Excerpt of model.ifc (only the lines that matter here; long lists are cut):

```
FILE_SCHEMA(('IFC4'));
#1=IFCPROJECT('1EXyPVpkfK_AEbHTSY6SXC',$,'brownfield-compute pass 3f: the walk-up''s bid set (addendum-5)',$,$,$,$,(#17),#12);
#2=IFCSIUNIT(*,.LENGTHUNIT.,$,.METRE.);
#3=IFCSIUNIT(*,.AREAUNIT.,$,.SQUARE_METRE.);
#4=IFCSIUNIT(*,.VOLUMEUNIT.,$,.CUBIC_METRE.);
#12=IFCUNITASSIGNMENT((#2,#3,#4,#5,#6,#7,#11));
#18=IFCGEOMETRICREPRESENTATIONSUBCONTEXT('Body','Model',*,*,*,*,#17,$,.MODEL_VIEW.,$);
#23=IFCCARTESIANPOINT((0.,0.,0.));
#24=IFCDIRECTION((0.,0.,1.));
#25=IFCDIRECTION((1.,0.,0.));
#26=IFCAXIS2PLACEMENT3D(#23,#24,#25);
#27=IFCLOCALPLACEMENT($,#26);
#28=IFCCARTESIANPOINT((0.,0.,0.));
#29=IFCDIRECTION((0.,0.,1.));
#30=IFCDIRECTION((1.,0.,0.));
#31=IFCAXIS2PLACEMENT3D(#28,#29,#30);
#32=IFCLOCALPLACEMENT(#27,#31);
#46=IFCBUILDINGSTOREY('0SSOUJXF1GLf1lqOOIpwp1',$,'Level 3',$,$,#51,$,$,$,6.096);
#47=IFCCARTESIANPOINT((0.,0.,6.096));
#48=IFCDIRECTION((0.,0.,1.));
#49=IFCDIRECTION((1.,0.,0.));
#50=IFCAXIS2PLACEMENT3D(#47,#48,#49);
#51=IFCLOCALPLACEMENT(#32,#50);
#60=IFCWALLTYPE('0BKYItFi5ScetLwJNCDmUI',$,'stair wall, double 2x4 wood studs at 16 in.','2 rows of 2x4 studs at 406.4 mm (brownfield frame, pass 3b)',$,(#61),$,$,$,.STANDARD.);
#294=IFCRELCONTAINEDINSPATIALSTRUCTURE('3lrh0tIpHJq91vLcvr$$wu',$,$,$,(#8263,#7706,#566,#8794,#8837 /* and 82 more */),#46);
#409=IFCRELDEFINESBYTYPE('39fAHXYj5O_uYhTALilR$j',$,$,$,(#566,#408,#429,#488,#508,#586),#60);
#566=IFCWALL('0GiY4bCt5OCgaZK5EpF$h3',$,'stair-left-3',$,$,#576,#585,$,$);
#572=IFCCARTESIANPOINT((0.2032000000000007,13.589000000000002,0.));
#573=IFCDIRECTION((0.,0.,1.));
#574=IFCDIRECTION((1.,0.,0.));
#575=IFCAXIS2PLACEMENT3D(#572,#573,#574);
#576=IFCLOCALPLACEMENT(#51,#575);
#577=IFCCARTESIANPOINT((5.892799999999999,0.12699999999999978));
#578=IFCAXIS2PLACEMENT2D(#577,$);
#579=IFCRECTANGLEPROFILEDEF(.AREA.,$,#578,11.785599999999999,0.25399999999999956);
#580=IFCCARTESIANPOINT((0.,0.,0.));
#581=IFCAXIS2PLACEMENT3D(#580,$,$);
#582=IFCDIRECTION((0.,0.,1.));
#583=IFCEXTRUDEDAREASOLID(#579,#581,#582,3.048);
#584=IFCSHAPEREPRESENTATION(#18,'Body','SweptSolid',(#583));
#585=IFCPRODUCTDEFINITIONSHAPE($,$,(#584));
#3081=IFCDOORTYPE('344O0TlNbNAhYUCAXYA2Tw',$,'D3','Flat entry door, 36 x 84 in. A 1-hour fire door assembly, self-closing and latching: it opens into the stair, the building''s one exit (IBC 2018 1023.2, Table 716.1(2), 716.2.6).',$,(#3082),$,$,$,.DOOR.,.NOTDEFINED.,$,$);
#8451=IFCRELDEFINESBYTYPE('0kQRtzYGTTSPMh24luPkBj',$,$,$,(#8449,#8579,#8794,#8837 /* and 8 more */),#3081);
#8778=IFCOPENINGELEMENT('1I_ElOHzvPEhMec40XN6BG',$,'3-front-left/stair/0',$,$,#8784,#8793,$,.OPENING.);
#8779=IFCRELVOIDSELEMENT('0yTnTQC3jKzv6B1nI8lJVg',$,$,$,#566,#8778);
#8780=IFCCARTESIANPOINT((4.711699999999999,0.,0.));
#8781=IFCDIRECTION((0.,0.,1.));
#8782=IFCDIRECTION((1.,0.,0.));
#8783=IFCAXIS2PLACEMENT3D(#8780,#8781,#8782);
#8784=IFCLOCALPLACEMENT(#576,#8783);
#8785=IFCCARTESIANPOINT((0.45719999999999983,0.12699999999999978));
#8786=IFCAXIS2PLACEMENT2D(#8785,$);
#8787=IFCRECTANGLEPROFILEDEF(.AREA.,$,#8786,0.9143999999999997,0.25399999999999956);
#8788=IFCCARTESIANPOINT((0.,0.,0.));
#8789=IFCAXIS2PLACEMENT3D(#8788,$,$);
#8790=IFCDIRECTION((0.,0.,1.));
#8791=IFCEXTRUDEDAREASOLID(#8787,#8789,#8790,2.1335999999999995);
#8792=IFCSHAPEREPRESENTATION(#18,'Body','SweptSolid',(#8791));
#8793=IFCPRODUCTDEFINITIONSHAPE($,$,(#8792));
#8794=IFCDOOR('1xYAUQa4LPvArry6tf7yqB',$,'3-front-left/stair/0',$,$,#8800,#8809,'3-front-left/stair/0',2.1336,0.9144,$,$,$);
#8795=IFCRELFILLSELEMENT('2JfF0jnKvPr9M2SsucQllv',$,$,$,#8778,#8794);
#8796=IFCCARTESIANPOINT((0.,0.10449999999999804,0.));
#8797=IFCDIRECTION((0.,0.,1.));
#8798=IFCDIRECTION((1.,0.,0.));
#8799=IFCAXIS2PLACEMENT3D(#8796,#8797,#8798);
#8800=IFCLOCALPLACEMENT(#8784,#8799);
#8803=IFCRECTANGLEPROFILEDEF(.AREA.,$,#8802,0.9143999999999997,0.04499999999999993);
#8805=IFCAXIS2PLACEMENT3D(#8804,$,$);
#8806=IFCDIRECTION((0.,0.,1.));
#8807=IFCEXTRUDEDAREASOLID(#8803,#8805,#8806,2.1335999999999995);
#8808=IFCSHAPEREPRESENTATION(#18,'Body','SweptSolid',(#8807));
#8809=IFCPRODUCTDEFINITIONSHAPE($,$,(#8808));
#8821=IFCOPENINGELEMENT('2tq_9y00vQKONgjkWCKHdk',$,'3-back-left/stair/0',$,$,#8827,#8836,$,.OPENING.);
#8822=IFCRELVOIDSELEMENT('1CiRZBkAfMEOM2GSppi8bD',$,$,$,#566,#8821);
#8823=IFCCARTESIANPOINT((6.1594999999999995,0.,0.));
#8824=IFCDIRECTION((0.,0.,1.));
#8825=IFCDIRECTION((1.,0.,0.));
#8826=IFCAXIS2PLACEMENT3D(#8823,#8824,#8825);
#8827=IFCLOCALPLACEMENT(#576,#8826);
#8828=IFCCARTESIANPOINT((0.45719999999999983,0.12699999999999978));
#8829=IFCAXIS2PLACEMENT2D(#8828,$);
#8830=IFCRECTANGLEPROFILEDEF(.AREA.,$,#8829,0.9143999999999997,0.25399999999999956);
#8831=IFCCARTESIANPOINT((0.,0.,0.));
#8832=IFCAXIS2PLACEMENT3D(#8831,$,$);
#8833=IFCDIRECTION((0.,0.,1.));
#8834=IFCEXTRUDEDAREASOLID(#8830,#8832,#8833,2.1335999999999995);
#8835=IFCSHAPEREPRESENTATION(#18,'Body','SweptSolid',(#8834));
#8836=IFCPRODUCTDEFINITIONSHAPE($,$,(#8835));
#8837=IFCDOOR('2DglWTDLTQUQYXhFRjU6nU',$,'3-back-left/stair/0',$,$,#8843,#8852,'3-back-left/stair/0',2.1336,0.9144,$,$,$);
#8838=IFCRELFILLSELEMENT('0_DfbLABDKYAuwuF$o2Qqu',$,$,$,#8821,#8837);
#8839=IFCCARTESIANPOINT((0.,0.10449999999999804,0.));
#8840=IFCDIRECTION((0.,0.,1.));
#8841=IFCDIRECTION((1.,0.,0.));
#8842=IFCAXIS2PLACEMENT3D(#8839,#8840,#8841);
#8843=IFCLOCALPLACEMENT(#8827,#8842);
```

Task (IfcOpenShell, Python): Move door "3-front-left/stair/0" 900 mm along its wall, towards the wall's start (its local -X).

```python
import ifcopenshell
import ifcopenshell.api.geometry
import ifcopenshell.util.placement
import ifcopenshell.util.unit

model = ifcopenshell.open("model.ifc")
unit_scale = ifcopenshell.util.unit.calculate_unit_scale(model)

door = model.by_guid("1xYAUQa4LPvArry6tf7yqB")
opening = door.FillsVoids[0].RelatingOpeningElement
wall = opening.VoidsElements[0].RelatingBuildingElement

wall_matrix = ifcopenshell.util.placement.get_local_placement(wall.ObjectPlacement)
shift = wall_matrix[:3, 0] * -0.9 / unit_scale
before = ifcopenshell.util.placement.get_local_placement(door.ObjectPlacement)[:3, 3].copy()

# The door is placed relative to its opening, so it follows when the opening moves.
matrix = ifcopenshell.util.placement.get_local_placement(opening.ObjectPlacement)
matrix[:3, 3] += shift
ifcopenshell.api.geometry.edit_object_placement(
    model, product=opening, matrix=matrix, is_si=False, should_transform_children=True
)

after = ifcopenshell.util.placement.get_local_placement(door.ObjectPlacement)[:3, 3]
print("door moved by", (after - before).round(3) + 0.0)

model.write("model_rev.ifc")
```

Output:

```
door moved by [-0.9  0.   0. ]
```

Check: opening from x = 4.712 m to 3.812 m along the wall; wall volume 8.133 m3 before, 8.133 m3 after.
